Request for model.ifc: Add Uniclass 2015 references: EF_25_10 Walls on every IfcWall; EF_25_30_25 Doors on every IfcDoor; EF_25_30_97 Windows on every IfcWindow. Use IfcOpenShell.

First a look at what the model holds.

```python
import ifcopenshell

model = ifcopenshell.open("model.ifc")
print(model.schema)
print("classifications:", [c.Name for c in model.by_type("IfcClassification")])
for ifc_class in ("IfcDoor", "IfcRoof", "IfcStair", "IfcWall", "IfcWindow"):
    print(ifc_class, len(model.by_type(ifc_class)))
```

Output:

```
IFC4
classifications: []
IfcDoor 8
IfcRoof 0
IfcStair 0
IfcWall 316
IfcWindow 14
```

```python
import ifcopenshell
import ifcopenshell.api.classification

model = ifcopenshell.open("model.ifc")

system = ifcopenshell.api.classification.add_classification(model, classification="Uniclass 2015")

codes = {
    "IfcWall": ("EF_25_10", "Walls"),
    "IfcDoor": ("EF_25_30_25", "Doors"),
    "IfcWindow": ("EF_25_30_97", "Windows"),
}
for ifc_class, (code, name) in codes.items():
    products = model.by_type(ifc_class)
    ifcopenshell.api.classification.add_reference(
        model, products=products, classification=system, identification=code, name=name
    )
    print(code, len(products))

model.write("model_rev.ifc")
```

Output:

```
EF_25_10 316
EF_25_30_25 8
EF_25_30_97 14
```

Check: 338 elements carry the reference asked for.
